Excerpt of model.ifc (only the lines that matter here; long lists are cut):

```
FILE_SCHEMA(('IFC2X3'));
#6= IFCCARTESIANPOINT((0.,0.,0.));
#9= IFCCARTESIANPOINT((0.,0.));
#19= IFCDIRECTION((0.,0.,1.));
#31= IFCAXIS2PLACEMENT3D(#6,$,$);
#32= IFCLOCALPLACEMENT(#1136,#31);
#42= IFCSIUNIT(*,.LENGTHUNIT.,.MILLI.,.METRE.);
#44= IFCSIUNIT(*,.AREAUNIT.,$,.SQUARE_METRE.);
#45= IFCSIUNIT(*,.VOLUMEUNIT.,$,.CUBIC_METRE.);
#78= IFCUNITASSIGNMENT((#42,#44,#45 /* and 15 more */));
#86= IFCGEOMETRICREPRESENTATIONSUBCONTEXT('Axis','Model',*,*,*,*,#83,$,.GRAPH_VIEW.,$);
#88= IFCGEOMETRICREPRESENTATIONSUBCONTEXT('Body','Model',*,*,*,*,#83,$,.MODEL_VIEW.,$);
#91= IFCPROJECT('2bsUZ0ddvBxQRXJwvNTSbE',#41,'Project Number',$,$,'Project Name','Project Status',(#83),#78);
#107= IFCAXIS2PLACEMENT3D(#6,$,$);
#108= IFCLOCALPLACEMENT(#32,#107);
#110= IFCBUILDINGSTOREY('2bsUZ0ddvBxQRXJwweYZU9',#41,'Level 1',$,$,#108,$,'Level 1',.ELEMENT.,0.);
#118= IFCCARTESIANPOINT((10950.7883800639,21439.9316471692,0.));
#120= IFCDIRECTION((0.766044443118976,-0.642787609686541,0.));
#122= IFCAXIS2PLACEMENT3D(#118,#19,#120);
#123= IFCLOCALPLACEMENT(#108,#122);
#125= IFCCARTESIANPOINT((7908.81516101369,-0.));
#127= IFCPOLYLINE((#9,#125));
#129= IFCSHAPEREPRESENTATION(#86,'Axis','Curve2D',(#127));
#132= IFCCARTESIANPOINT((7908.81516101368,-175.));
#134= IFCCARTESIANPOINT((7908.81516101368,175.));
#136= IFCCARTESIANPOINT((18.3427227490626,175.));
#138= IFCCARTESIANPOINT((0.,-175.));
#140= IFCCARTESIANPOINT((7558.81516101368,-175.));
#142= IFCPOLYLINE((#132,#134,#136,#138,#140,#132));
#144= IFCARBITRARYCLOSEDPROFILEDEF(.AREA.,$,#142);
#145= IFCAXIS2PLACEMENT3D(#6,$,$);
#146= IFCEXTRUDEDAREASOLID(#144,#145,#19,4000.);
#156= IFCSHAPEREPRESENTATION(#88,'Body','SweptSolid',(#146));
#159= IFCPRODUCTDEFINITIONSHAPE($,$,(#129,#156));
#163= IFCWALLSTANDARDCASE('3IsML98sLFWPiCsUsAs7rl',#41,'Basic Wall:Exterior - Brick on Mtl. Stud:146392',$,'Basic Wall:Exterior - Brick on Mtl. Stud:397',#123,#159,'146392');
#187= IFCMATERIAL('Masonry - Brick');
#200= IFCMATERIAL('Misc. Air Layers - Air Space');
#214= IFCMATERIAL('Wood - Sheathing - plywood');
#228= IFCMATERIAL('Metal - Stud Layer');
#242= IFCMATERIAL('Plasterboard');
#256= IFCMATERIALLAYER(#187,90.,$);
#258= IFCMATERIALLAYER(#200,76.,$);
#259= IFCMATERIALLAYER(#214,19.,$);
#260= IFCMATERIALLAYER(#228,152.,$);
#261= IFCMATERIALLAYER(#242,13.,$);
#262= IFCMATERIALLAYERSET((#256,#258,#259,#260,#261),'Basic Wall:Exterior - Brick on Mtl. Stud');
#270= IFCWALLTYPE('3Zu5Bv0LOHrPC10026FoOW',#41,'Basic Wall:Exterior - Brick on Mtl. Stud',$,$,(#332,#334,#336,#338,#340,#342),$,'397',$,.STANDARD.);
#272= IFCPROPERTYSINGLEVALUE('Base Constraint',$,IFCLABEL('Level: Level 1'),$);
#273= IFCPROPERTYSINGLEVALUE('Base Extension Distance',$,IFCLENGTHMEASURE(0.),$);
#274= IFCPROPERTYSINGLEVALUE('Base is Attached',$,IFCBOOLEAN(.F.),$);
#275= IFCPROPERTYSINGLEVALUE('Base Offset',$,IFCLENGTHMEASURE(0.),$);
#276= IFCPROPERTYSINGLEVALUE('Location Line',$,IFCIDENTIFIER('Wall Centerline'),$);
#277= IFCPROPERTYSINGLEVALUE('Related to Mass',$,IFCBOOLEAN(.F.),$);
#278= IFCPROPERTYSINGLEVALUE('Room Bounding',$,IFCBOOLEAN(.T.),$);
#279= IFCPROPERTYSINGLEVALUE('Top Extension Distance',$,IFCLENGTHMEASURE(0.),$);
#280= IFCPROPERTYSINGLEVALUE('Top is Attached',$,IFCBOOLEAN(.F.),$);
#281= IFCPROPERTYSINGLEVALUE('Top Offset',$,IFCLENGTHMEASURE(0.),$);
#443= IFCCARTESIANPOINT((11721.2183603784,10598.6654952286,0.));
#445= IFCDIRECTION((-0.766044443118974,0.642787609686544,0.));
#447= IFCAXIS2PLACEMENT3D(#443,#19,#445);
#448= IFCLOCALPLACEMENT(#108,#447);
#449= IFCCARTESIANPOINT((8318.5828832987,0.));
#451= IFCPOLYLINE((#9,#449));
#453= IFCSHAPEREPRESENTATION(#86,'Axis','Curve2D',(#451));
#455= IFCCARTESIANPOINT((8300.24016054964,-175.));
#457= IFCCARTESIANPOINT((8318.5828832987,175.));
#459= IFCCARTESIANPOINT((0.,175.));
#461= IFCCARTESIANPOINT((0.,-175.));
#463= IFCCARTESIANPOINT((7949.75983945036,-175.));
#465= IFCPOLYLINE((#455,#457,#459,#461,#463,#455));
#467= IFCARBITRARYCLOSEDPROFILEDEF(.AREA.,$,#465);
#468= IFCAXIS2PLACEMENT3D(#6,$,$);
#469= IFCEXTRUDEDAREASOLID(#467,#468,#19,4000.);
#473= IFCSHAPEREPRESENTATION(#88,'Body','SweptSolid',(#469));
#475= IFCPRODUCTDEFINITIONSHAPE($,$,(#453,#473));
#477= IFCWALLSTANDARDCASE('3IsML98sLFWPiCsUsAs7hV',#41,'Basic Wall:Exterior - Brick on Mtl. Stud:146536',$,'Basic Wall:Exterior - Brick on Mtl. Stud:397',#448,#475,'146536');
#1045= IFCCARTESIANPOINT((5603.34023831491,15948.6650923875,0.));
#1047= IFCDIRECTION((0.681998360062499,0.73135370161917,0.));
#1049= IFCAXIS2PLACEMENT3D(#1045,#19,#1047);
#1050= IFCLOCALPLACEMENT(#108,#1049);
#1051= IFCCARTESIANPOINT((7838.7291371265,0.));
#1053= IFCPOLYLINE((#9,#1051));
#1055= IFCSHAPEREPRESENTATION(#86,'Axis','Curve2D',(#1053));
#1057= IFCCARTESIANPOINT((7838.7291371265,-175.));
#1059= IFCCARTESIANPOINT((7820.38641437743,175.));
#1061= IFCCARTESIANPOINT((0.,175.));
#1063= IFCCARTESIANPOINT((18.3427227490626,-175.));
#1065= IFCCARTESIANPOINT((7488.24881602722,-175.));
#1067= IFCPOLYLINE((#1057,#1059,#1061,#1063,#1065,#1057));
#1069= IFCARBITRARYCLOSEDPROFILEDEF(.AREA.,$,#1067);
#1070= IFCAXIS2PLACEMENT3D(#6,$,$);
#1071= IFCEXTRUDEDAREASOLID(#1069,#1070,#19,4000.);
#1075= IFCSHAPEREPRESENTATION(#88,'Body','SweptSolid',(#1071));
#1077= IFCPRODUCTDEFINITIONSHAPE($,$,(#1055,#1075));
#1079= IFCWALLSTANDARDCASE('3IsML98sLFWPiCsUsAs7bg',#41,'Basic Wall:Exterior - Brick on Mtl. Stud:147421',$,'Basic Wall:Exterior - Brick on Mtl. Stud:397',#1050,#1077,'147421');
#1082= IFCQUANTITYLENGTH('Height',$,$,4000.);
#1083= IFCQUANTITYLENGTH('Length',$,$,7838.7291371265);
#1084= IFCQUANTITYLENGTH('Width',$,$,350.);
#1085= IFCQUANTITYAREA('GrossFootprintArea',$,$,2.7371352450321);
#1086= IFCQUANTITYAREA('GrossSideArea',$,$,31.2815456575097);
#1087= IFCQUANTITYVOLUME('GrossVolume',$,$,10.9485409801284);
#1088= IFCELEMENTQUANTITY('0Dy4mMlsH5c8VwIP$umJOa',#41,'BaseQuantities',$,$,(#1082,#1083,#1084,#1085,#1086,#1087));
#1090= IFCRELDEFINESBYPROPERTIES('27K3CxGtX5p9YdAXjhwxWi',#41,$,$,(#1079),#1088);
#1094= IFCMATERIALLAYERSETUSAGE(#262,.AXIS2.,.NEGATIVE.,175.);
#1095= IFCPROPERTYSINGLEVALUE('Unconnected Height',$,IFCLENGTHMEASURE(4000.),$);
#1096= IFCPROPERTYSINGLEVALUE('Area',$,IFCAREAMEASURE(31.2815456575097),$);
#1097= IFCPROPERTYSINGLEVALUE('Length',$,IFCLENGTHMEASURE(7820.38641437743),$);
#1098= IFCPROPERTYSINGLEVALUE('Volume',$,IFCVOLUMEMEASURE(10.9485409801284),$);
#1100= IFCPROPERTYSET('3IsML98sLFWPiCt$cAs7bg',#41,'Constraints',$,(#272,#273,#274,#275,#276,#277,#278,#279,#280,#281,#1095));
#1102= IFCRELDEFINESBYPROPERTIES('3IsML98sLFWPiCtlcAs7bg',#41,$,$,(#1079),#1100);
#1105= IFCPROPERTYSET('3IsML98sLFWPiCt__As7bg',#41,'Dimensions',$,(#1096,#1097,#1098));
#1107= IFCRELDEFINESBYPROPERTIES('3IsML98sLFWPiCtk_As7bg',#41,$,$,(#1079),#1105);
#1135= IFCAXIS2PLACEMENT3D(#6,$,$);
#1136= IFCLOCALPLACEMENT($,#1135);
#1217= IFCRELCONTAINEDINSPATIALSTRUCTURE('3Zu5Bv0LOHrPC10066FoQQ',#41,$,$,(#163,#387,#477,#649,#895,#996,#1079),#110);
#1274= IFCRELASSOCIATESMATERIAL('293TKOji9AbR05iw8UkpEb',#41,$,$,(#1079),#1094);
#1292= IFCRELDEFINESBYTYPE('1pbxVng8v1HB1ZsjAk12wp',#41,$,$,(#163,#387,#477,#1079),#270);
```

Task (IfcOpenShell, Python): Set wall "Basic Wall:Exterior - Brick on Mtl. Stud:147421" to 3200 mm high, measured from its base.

```python
import ifcopenshell
import ifcopenshell.api.pset
import ifcopenshell.geom
import ifcopenshell.util.element
import ifcopenshell.util.representation
import ifcopenshell.util.shape
import ifcopenshell.util.unit

model = ifcopenshell.open("model.ifc")
unit_scale = ifcopenshell.util.unit.calculate_unit_scale(model)
area_scale = ifcopenshell.util.unit.calculate_unit_scale(model, "AREAUNIT")
volume_scale = ifcopenshell.util.unit.calculate_unit_scale(model, "VOLUMEUNIT")
settings = ifcopenshell.geom.settings()


def volume(element):
    """Net volume in cubic metres, openings subtracted."""
    shape = ifcopenshell.geom.create_shape(settings, element)
    return ifcopenshell.util.shape.get_volume(shape.geometry)


wall = model.by_guid("3IsML98sLFWPiCsUsAs7bg")
before = volume(wall)

body = ifcopenshell.util.representation.get_representation(wall, "Model", "Body")
solid = body.Items[0]
old_height = solid.Depth
solid.Depth = 3200.0
after = volume(wall)
thickness = 0.35  # wall thickness in metres

# Update the stored height, areas and volumes.
qto = model.by_id(ifcopenshell.util.element.get_pset(wall, "BaseQuantities", should_inherit=False)["id"])
ifcopenshell.api.pset.edit_qto(model, qto=qto, properties={
    "Height": solid.Depth,
    "GrossSideArea": ifcopenshell.util.element.get_pset(wall, "BaseQuantities", "GrossSideArea") * solid.Depth / old_height,
    "GrossVolume": ifcopenshell.util.element.get_pset(wall, "BaseQuantities", "GrossVolume") * solid.Depth / old_height,
})
pset = model.by_id(ifcopenshell.util.element.get_pset(wall, "Constraints", should_inherit=False)["id"])
ifcopenshell.api.pset.edit_pset(model, pset=pset, properties={
    "Unconnected Height": model.create_entity("IfcLengthMeasure", solid.Depth),
})
pset = model.by_id(ifcopenshell.util.element.get_pset(wall, "Dimensions", should_inherit=False)["id"])
ifcopenshell.api.pset.edit_pset(model, pset=pset, properties={
    "Area": model.create_entity("IfcAreaMeasure", after / thickness / area_scale),
    "Volume": model.create_entity("IfcVolumeMeasure", after / volume_scale),
})

print(f"height {old_height:g} -> {solid.Depth:g}, volume {before:.3f} -> {after:.3f} m3")

model.write("model_v2.ifc")
```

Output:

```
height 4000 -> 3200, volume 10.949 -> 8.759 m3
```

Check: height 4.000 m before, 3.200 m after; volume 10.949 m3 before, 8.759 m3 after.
